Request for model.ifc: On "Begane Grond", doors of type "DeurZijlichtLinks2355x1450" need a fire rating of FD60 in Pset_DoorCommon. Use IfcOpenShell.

First a look at what the model holds.

```python
import ifcopenshell
import ifcopenshell.util.element

model = ifcopenshell.open("model.ifc")
print(model.schema)
storey = next(s for s in model.by_type("IfcBuildingStorey") if s.Name == "Begane Grond")
doors = [e for e in ifcopenshell.util.element.get_decomposition(storey) if e.is_a("IfcDoor")]
seen = {}
for e in doors:
    element_type = ifcopenshell.util.element.get_type(e)
    key = (element_type.Name if element_type != e and element_type else None, ifcopenshell.util.element.get_pset(e, "Pset_DoorCommon", "FireRating"))
    seen[key] = seen.get(key, 0) + 1
for (name, value), count in sorted(seen.items(), key=str):
    print(count, "x", name, "|", value)
```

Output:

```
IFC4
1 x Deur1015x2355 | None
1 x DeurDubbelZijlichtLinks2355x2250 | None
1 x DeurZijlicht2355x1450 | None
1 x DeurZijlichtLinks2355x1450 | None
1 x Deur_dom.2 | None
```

```python
import ifcopenshell
import ifcopenshell.api.pset
import ifcopenshell.util.element

model = ifcopenshell.open("model.ifc")

storey = next(s for s in model.by_type("IfcBuildingStorey") if s.Name == "Begane Grond")
doors = [e for e in ifcopenshell.util.element.get_decomposition(storey) if e.is_a("IfcDoor")]

count = 0
for e in doors:
    element_type = ifcopenshell.util.element.get_type(e)
    if element_type in (None, e) or element_type.Name != "DeurZijlichtLinks2355x1450":
        continue
    # add_pset returns the element's existing set when there is one.
    pset = ifcopenshell.api.pset.add_pset(model, product=e, name="Pset_DoorCommon")
    ifcopenshell.api.pset.edit_pset(model, pset=pset, properties={"FireRating": "FD60"})
    count += 1

print(count, "doors updated")

model.write("model_rev.ifc")
```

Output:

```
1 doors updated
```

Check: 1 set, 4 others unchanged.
